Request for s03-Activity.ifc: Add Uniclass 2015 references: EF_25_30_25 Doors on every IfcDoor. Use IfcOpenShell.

First a look at what the model holds.

```python
import ifcopenshell

model = ifcopenshell.open("s03-Activity.ifc")
print(model.schema)
print("classifications:", [c.Name for c in model.by_type("IfcClassification")])
for ifc_class in ("IfcDoor", "IfcRoof", "IfcStair", "IfcWall", "IfcWindow"):
    print(ifc_class, len(model.by_type(ifc_class)))
```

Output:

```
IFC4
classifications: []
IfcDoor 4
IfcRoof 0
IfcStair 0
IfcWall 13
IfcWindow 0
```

```python
import ifcopenshell
import ifcopenshell.api.classification

model = ifcopenshell.open("s03-Activity.ifc")

system = ifcopenshell.api.classification.add_classification(model, classification="Uniclass 2015")

codes = {
    "IfcDoor": ("EF_25_30_25", "Doors"),
}
for ifc_class, (code, name) in codes.items():
    products = model.by_type(ifc_class)
    ifcopenshell.api.classification.add_reference(
        model, products=products, classification=system, identification=code, name=name
    )
    print(code, len(products))

model.write("s03-Activity_edited.ifc")
```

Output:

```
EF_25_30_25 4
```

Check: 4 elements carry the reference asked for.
